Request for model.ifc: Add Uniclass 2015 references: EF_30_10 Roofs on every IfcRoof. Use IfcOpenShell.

First a look at what the model holds.

```python
import ifcopenshell

model = ifcopenshell.open("model.ifc")
print(model.schema)
print("classifications:", [c.Name for c in model.by_type("IfcClassification")])
for ifc_class in ("IfcDoor", "IfcRoof", "IfcStair", "IfcWall", "IfcWindow"):
    print(ifc_class, len(model.by_type(ifc_class)))
```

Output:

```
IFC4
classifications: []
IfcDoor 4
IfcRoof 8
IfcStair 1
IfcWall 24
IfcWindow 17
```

```python
import ifcopenshell
import ifcopenshell.api.classification

model = ifcopenshell.open("model.ifc")

system = ifcopenshell.api.classification.add_classification(model, classification="Uniclass 2015")

codes = {
    "IfcRoof": ("EF_30_10", "Roofs"),
}
for ifc_class, (code, name) in codes.items():
    products = model.by_type(ifc_class)
    ifcopenshell.api.classification.add_reference(
        model, products=products, classification=system, identification=code, name=name
    )
    print(code, len(products))

model.write("model_v2.ifc")
```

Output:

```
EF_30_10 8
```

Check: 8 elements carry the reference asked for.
